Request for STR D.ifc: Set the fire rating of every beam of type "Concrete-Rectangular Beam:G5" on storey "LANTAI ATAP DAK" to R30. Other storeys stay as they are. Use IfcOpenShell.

First a look at what the model holds.

```python
import ifcopenshell
import ifcopenshell.util.element

model = ifcopenshell.open("STR D.ifc")
print(model.schema)
storey = next(s for s in model.by_type("IfcBuildingStorey") if s.Name == "LANTAI ATAP DAK")
beams = [e for e in ifcopenshell.util.element.get_decomposition(storey) if e.is_a("IfcBeam")]
seen = {}
for e in beams:
    element_type = ifcopenshell.util.element.get_type(e)
    key = (element_type.Name if element_type != e and element_type else None, ifcopenshell.util.element.get_pset(e, "Pset_BeamCommon", "FireRating"))
    seen[key] = seen.get(key, 0) + 1
for (name, value), count in sorted(seen.items(), key=str):
    print(count, "x", name, "|", value)
```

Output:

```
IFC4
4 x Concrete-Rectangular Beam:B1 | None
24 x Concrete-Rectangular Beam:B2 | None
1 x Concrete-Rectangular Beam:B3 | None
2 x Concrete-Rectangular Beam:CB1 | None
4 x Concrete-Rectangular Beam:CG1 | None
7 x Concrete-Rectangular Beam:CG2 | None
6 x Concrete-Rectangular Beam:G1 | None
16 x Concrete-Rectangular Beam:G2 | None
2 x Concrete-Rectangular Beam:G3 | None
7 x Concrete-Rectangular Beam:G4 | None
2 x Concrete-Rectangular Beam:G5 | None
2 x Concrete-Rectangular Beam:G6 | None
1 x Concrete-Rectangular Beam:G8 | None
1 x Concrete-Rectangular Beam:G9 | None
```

```python
import ifcopenshell
import ifcopenshell.api.pset
import ifcopenshell.util.element

model = ifcopenshell.open("STR D.ifc")

storey = next(s for s in model.by_type("IfcBuildingStorey") if s.Name == "LANTAI ATAP DAK")
beams = [e for e in ifcopenshell.util.element.get_decomposition(storey) if e.is_a("IfcBeam")]

count = 0
for e in beams:
    element_type = ifcopenshell.util.element.get_type(e)
    if element_type in (None, e) or element_type.Name != "Concrete-Rectangular Beam:G5":
        continue
    # add_pset returns the element's existing set when there is one.
    pset = ifcopenshell.api.pset.add_pset(model, product=e, name="Pset_BeamCommon")
    ifcopenshell.api.pset.edit_pset(model, pset=pset, properties={"FireRating": "R30"})
    count += 1

print(count, "beams updated")

model.write("STR D_edited.ifc")
```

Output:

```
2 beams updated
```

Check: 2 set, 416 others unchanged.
